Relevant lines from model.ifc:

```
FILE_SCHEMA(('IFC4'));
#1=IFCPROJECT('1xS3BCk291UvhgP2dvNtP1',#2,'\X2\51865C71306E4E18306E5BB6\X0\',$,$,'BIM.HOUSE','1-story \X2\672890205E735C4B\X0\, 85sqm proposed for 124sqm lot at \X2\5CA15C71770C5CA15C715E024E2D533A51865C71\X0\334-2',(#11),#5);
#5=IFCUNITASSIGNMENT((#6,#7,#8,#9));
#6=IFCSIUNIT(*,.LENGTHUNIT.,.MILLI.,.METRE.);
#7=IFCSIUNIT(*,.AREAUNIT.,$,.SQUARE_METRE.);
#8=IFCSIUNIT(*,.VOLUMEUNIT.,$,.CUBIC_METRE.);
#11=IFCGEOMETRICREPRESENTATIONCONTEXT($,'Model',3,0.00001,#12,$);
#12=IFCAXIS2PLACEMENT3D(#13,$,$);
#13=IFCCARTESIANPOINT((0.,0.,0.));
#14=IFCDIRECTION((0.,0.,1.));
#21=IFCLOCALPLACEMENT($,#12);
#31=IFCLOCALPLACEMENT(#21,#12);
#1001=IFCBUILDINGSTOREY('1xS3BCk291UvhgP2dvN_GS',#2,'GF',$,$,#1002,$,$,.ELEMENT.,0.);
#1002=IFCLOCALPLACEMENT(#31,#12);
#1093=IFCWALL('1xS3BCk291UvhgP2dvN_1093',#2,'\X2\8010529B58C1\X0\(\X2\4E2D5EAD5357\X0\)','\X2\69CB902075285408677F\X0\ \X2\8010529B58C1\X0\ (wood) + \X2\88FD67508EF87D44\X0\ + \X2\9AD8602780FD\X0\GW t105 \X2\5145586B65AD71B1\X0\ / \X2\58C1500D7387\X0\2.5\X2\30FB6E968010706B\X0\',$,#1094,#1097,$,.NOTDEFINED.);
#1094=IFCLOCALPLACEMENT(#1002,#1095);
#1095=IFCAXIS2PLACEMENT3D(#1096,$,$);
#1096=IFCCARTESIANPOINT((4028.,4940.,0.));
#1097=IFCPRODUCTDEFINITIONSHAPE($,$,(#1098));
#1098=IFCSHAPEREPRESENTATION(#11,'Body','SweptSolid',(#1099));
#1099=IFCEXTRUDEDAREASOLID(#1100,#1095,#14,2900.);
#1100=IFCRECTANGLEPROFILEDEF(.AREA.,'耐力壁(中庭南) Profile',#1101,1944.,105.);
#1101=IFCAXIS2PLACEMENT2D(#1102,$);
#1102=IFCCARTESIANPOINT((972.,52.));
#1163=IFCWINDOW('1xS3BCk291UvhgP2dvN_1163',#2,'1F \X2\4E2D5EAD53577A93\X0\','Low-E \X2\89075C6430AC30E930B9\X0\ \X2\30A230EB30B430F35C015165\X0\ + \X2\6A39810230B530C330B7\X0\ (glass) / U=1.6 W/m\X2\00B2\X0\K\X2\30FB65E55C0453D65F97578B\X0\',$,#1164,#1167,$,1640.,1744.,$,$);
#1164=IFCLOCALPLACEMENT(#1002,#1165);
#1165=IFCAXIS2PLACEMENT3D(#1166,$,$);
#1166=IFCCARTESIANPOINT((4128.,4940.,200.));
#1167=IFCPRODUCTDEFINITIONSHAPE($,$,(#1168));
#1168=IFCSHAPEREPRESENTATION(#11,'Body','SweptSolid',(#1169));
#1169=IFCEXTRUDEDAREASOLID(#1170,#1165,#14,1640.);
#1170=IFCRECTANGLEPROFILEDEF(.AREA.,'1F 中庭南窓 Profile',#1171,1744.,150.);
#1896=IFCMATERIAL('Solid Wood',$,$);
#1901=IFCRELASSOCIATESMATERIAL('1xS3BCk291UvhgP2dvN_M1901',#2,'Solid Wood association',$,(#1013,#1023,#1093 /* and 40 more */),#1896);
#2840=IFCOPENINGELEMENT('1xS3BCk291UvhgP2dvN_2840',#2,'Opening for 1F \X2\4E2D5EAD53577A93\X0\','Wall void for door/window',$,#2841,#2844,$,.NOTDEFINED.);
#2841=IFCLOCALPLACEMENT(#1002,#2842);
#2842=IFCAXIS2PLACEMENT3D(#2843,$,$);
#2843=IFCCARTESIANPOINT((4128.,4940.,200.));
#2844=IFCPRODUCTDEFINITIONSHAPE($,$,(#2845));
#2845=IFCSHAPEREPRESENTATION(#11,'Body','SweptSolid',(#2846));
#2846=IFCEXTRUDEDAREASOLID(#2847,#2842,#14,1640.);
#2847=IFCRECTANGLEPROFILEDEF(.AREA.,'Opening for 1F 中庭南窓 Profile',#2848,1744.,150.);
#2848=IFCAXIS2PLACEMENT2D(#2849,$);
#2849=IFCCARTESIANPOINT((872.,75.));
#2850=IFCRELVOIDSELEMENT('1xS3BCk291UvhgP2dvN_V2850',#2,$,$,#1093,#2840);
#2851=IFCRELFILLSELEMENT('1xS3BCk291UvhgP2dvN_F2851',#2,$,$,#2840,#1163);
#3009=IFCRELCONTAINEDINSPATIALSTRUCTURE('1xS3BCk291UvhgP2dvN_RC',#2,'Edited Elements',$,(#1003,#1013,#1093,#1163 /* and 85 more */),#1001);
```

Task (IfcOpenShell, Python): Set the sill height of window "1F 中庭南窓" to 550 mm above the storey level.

```python
import numpy as np
import ifcopenshell
import ifcopenshell.api.geometry
import ifcopenshell.geom
import ifcopenshell.util.element
import ifcopenshell.util.placement
import ifcopenshell.util.shape
import ifcopenshell.util.unit

model = ifcopenshell.open("model.ifc")
unit_scale = ifcopenshell.util.unit.calculate_unit_scale(model)

window = model.by_guid("1xS3BCk291UvhgP2dvN_1163")
opening = window.FillsVoids[0].RelatingOpeningElement
storey = ifcopenshell.util.element.get_container(window, ifc_class="IfcBuildingStorey")
level = ifcopenshell.util.placement.get_local_placement(storey.ObjectPlacement)[2, 3]

# The opening's origin need not be at the sill, so measure its lowest point.
shape = ifcopenshell.geom.create_shape(ifcopenshell.geom.settings(), opening)
bottom = ifcopenshell.util.shape.get_shape_bottom_elevation(shape, shape.geometry) / unit_scale
dz = level + 0.55 / unit_scale - bottom

shift = np.array([0.0, 0.0, dz])
# The window is not placed relative to its opening, so move both.
for product in (opening, window):
    matrix = ifcopenshell.util.placement.get_local_placement(product.ObjectPlacement)
    matrix[:3, 3] += shift
    ifcopenshell.api.geometry.edit_object_placement(model, product=product, matrix=matrix, is_si=False)

print(f"moved by {dz * unit_scale:+.3f} m")

model.write("model_updated.ifc")
```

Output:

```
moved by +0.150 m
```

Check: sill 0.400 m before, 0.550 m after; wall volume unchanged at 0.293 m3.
